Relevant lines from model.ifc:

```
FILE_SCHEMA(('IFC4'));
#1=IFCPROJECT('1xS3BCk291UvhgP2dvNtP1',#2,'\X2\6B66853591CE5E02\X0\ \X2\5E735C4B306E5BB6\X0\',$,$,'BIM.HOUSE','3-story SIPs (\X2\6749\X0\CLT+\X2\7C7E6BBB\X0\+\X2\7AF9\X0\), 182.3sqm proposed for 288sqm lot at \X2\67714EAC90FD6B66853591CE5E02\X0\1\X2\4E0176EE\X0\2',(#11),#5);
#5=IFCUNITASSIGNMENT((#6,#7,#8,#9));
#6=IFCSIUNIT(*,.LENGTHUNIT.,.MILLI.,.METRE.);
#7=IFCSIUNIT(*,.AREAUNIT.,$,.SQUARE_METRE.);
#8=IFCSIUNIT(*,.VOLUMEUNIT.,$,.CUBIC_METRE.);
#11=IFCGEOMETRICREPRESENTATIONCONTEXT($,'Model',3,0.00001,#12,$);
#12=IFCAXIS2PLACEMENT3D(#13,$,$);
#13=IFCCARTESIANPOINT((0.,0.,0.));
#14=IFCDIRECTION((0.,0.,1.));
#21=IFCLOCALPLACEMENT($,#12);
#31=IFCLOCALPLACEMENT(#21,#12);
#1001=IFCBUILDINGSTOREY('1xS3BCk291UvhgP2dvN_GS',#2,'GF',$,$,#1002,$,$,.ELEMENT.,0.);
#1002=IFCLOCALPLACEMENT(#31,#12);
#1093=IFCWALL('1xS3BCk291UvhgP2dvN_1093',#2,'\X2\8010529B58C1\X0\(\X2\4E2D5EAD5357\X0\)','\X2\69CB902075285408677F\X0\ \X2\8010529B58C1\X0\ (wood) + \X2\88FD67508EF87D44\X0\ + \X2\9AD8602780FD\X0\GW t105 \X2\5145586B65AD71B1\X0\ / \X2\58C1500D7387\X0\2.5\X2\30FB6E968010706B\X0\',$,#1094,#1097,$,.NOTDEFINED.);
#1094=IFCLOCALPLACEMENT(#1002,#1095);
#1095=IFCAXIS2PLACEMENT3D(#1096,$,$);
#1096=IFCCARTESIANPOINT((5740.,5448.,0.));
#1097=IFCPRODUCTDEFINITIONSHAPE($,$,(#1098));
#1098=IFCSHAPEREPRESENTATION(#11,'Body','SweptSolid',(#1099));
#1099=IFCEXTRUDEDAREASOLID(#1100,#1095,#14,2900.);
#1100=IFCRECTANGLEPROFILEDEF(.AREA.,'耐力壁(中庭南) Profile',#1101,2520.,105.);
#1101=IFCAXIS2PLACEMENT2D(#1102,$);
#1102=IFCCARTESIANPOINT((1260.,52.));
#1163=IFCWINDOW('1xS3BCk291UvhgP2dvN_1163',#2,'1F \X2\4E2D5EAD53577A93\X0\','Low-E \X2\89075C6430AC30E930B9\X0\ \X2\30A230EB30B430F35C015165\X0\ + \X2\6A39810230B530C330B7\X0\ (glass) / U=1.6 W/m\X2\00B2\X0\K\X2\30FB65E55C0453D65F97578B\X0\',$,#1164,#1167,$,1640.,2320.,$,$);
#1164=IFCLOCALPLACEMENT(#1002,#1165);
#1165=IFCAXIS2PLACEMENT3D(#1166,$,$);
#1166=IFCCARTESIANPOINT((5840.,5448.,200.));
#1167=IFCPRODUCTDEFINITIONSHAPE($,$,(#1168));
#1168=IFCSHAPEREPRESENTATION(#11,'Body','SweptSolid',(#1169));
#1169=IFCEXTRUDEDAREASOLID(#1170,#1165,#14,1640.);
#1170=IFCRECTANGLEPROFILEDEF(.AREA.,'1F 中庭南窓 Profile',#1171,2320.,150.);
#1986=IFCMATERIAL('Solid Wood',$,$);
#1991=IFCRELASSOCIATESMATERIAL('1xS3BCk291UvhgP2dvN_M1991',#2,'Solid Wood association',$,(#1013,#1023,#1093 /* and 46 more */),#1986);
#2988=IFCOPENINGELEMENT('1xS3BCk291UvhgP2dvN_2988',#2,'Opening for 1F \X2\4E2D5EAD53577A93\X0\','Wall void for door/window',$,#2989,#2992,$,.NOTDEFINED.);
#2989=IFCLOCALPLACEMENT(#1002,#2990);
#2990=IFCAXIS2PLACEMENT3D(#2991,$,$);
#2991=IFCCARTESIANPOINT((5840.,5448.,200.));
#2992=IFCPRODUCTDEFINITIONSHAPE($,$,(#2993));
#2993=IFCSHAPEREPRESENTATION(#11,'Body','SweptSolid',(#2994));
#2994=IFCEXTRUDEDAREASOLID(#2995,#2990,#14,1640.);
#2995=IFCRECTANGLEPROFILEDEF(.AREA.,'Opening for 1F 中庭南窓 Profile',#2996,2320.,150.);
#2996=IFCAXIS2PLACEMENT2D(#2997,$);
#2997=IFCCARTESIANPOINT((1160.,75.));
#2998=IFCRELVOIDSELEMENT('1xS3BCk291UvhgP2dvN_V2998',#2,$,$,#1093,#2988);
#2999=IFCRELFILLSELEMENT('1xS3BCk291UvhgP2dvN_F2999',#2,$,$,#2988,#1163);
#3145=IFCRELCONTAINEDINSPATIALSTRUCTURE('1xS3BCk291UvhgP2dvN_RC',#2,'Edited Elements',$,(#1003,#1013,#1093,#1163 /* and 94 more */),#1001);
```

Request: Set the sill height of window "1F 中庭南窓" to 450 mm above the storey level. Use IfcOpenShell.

```python
import numpy as np
import ifcopenshell
import ifcopenshell.api.geometry
import ifcopenshell.geom
import ifcopenshell.util.element
import ifcopenshell.util.placement
import ifcopenshell.util.shape
import ifcopenshell.util.unit

model = ifcopenshell.open("model.ifc")
unit_scale = ifcopenshell.util.unit.calculate_unit_scale(model)

window = model.by_guid("1xS3BCk291UvhgP2dvN_1163")
opening = window.FillsVoids[0].RelatingOpeningElement
storey = ifcopenshell.util.element.get_container(window, ifc_class="IfcBuildingStorey")
level = ifcopenshell.util.placement.get_local_placement(storey.ObjectPlacement)[2, 3]

# The opening's origin need not be at the sill, so measure its lowest point.
shape = ifcopenshell.geom.create_shape(ifcopenshell.geom.settings(), opening)
bottom = ifcopenshell.util.shape.get_shape_bottom_elevation(shape, shape.geometry) / unit_scale
dz = level + 450.0 - bottom

shift = np.array([0.0, 0.0, dz])
# The window is not placed relative to its opening, so move both.
for product in (opening, window):
    matrix = ifcopenshell.util.placement.get_local_placement(product.ObjectPlacement)
    matrix[:3, 3] += shift
    ifcopenshell.api.geometry.edit_object_placement(model, product=product, matrix=matrix, is_si=False)

print(f"moved by {dz * unit_scale:+.3f} m")

model.write("model_v2.ifc")
```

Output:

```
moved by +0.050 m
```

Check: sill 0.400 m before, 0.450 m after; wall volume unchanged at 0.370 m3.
